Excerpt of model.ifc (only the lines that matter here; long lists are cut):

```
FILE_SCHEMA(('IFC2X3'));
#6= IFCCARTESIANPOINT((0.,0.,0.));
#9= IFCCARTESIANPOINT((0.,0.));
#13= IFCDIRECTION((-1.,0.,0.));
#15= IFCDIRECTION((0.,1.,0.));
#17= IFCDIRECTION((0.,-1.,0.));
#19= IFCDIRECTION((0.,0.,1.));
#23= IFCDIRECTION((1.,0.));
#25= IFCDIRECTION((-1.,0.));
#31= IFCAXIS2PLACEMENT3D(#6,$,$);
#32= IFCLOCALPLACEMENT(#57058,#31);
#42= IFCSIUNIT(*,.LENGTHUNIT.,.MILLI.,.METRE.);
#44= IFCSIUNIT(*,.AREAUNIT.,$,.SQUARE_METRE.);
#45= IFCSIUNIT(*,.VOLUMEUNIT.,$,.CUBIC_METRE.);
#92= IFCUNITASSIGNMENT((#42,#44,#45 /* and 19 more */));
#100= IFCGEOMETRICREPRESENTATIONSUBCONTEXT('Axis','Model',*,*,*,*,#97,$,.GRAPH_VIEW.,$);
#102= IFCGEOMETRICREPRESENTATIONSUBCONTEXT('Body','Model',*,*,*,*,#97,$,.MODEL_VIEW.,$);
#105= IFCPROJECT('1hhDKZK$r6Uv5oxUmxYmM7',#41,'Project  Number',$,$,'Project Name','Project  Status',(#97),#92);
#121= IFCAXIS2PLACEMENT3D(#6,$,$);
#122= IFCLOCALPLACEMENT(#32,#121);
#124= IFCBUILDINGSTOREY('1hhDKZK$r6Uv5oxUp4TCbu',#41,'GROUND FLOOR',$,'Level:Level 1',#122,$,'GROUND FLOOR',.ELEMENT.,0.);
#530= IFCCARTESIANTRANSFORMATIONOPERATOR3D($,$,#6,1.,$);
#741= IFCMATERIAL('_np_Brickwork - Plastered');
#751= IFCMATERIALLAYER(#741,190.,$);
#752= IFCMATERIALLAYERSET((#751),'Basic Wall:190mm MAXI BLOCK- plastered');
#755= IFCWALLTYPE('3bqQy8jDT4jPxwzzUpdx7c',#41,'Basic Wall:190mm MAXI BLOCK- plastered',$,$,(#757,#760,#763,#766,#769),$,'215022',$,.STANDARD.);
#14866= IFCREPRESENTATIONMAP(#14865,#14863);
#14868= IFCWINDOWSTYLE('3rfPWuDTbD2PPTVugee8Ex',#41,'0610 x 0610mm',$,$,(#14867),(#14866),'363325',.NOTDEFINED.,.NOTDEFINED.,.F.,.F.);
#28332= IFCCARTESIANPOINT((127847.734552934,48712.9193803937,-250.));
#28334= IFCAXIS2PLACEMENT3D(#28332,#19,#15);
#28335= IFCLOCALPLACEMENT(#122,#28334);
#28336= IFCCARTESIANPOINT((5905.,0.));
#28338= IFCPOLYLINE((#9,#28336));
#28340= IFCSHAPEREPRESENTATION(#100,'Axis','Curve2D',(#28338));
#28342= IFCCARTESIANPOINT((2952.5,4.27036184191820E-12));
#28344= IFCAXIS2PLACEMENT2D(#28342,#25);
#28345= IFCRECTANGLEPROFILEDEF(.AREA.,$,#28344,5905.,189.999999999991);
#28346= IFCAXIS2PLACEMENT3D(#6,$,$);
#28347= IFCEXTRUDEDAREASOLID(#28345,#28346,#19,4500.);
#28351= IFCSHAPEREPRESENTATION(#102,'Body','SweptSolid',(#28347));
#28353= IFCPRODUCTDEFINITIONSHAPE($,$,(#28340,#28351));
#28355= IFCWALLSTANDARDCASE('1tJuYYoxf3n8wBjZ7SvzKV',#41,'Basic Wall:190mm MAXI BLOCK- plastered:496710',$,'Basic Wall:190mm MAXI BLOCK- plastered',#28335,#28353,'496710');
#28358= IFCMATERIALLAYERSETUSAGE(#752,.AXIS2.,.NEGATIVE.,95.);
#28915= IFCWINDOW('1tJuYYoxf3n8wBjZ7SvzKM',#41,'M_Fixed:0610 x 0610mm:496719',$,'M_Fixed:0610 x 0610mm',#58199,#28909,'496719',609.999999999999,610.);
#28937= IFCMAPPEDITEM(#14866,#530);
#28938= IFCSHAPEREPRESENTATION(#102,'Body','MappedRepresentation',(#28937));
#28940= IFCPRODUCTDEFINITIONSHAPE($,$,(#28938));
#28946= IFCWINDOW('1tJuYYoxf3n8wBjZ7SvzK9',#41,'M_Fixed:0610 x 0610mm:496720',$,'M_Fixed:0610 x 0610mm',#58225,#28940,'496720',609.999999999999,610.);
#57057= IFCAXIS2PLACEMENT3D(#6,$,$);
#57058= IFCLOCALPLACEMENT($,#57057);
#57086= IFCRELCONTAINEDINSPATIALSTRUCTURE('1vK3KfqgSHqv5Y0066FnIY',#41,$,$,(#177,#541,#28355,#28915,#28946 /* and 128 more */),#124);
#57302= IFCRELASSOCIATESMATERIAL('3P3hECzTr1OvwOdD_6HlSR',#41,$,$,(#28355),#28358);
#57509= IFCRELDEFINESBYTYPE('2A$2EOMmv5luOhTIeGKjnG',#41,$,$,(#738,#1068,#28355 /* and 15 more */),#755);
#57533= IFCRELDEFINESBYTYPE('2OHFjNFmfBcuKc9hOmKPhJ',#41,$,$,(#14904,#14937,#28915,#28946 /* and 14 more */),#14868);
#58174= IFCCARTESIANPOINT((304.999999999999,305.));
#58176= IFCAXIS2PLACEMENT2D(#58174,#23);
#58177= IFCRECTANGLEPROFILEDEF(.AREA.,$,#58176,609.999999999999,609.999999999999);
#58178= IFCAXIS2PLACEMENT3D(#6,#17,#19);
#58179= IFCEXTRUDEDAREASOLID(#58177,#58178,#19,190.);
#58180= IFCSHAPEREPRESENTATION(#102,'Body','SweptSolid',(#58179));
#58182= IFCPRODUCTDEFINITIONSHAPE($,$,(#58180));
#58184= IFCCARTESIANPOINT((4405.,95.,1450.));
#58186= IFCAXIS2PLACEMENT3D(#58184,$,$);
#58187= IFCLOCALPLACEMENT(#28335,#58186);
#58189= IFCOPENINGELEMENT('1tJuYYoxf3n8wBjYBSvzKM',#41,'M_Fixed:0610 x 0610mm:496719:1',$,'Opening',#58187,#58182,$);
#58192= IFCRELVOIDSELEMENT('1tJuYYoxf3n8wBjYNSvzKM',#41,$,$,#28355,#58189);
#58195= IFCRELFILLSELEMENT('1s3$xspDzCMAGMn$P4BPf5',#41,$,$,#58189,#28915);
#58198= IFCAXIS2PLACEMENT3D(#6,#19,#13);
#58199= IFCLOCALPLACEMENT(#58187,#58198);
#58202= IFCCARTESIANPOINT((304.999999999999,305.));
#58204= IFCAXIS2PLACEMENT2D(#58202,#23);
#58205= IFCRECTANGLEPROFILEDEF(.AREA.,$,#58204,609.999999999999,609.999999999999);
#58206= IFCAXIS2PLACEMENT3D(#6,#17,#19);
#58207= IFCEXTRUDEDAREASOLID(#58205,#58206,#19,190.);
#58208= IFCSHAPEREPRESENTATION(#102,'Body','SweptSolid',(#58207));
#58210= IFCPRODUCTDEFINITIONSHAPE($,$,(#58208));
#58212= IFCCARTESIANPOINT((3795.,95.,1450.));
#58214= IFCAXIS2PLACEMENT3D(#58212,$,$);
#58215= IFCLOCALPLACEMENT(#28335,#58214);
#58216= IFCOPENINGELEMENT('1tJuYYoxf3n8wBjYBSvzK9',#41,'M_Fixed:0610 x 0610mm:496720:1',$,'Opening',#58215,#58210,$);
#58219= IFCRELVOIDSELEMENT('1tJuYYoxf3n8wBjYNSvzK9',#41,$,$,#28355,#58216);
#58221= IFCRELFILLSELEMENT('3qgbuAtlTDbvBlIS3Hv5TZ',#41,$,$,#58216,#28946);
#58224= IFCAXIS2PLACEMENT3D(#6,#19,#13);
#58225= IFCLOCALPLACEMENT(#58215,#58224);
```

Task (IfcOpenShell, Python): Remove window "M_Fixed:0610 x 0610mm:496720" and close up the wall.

```python
import ifcopenshell
import ifcopenshell.api.feature
import ifcopenshell.api.root
import ifcopenshell.geom
import ifcopenshell.util.shape

model = ifcopenshell.open("model.ifc")
settings = ifcopenshell.geom.settings()


def volume(element):
    """Net volume in cubic metres, openings subtracted."""
    shape = ifcopenshell.geom.create_shape(settings, element)
    return ifcopenshell.util.shape.get_volume(shape.geometry)


window = model.by_guid("1tJuYYoxf3n8wBjZ7SvzK9")
opening = window.FillsVoids[0].RelatingOpeningElement
wall = opening.VoidsElements[0].RelatingBuildingElement
before = volume(wall)

ifcopenshell.api.root.remove_product(model, product=window)
ifcopenshell.api.feature.remove_feature(model, feature=opening)

after = volume(wall)

print(f"wall volume {before:.3f} -> {after:.3f} m3")

model.write("model_updated.ifc")
```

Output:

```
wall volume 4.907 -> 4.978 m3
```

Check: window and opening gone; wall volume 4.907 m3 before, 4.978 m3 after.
